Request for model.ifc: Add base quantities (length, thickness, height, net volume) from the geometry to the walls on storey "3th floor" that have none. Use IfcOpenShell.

First a look at what the model holds.

```python
import ifcopenshell
import ifcopenshell.util.element
import ifcopenshell.util.unit

model = ifcopenshell.open("model.ifc")
print(model.schema)
for unit_type in ("LENGTHUNIT", "AREAUNIT", "VOLUMEUNIT"):
    print(unit_type, ifcopenshell.util.unit.calculate_unit_scale(model, unit_type))
storey = next(s for s in model.by_type("IfcBuildingStorey") if s.Name == "3th floor")
walls = [e for e in ifcopenshell.util.element.get_decomposition(storey) if e.is_a("IfcWall")]
for e in sorted(walls, key=lambda e: e.id()):
    print(e.id(), e.is_a(), e.Name, list(ifcopenshell.util.element.get_psets(e, qtos_only=True)), sep=" | ")
```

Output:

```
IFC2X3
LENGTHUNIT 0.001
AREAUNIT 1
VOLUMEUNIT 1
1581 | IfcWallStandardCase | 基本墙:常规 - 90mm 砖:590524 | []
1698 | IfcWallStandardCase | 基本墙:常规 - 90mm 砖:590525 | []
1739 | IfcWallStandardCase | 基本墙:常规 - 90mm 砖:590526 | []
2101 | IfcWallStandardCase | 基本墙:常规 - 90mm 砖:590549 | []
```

```python
import ifcopenshell
import ifcopenshell.api.pset
import ifcopenshell.geom
import ifcopenshell.util.element
import ifcopenshell.util.shape
import ifcopenshell.util.unit

model = ifcopenshell.open("model.ifc")
unit_scale = ifcopenshell.util.unit.calculate_unit_scale(model)
volume_scale = ifcopenshell.util.unit.calculate_unit_scale(model, "VOLUMEUNIT")
settings = ifcopenshell.geom.settings()

storey = next(s for s in model.by_type("IfcBuildingStorey") if s.Name == "3th floor")
walls = [e for e in ifcopenshell.util.element.get_decomposition(storey) if e.is_a("IfcWall")]

for e in sorted(walls, key=lambda e: e.id()):
    if ifcopenshell.util.element.get_psets(e, qtos_only=True, should_inherit=False):
        continue
    # Geometry comes back in metres, in the element's own axes.
    shape = ifcopenshell.geom.create_shape(settings, e)
    values = {
        "Length": ifcopenshell.util.shape.get_x(shape.geometry) / unit_scale,
        "Width": ifcopenshell.util.shape.get_y(shape.geometry) / unit_scale,
        "Height": ifcopenshell.util.shape.get_z(shape.geometry) / unit_scale,
        "NetVolume": ifcopenshell.util.shape.get_volume(shape.geometry) / volume_scale,
    }
    qto = ifcopenshell.api.pset.add_qto(model, product=e, name="BaseQuantities")
    ifcopenshell.api.pset.edit_qto(model, qto=qto, properties=values)
    print(e.id(), {k: round(v, 3) for k, v in values.items()})

model.write("model_updated.ifc")
```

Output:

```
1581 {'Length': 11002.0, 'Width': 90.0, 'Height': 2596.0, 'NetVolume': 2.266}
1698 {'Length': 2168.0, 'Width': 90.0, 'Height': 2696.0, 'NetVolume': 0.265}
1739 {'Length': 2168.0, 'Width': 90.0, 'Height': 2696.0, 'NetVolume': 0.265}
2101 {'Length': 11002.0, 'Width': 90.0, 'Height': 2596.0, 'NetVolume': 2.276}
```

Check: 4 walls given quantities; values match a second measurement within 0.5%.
